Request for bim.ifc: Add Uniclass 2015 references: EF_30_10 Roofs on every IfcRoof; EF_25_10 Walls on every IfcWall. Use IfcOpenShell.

First a look at what the model holds.

```python
import ifcopenshell

model = ifcopenshell.open("bim.ifc")
print(model.schema)
print("classifications:", [c.Name for c in model.by_type("IfcClassification")])
for ifc_class in ("IfcDoor", "IfcRoof", "IfcStair", "IfcWall", "IfcWindow"):
    print(ifc_class, len(model.by_type(ifc_class)))
```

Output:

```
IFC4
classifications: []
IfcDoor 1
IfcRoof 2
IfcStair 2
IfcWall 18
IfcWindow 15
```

```python
import ifcopenshell
import ifcopenshell.api.classification

model = ifcopenshell.open("bim.ifc")

system = ifcopenshell.api.classification.add_classification(model, classification="Uniclass 2015")

codes = {
    "IfcRoof": ("EF_30_10", "Roofs"),
    "IfcWall": ("EF_25_10", "Walls"),
}
for ifc_class, (code, name) in codes.items():
    products = model.by_type(ifc_class)
    ifcopenshell.api.classification.add_reference(
        model, products=products, classification=system, identification=code, name=name
    )
    print(code, len(products))

model.write("bim_edited.ifc")
```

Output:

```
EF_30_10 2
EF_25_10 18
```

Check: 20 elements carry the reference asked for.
